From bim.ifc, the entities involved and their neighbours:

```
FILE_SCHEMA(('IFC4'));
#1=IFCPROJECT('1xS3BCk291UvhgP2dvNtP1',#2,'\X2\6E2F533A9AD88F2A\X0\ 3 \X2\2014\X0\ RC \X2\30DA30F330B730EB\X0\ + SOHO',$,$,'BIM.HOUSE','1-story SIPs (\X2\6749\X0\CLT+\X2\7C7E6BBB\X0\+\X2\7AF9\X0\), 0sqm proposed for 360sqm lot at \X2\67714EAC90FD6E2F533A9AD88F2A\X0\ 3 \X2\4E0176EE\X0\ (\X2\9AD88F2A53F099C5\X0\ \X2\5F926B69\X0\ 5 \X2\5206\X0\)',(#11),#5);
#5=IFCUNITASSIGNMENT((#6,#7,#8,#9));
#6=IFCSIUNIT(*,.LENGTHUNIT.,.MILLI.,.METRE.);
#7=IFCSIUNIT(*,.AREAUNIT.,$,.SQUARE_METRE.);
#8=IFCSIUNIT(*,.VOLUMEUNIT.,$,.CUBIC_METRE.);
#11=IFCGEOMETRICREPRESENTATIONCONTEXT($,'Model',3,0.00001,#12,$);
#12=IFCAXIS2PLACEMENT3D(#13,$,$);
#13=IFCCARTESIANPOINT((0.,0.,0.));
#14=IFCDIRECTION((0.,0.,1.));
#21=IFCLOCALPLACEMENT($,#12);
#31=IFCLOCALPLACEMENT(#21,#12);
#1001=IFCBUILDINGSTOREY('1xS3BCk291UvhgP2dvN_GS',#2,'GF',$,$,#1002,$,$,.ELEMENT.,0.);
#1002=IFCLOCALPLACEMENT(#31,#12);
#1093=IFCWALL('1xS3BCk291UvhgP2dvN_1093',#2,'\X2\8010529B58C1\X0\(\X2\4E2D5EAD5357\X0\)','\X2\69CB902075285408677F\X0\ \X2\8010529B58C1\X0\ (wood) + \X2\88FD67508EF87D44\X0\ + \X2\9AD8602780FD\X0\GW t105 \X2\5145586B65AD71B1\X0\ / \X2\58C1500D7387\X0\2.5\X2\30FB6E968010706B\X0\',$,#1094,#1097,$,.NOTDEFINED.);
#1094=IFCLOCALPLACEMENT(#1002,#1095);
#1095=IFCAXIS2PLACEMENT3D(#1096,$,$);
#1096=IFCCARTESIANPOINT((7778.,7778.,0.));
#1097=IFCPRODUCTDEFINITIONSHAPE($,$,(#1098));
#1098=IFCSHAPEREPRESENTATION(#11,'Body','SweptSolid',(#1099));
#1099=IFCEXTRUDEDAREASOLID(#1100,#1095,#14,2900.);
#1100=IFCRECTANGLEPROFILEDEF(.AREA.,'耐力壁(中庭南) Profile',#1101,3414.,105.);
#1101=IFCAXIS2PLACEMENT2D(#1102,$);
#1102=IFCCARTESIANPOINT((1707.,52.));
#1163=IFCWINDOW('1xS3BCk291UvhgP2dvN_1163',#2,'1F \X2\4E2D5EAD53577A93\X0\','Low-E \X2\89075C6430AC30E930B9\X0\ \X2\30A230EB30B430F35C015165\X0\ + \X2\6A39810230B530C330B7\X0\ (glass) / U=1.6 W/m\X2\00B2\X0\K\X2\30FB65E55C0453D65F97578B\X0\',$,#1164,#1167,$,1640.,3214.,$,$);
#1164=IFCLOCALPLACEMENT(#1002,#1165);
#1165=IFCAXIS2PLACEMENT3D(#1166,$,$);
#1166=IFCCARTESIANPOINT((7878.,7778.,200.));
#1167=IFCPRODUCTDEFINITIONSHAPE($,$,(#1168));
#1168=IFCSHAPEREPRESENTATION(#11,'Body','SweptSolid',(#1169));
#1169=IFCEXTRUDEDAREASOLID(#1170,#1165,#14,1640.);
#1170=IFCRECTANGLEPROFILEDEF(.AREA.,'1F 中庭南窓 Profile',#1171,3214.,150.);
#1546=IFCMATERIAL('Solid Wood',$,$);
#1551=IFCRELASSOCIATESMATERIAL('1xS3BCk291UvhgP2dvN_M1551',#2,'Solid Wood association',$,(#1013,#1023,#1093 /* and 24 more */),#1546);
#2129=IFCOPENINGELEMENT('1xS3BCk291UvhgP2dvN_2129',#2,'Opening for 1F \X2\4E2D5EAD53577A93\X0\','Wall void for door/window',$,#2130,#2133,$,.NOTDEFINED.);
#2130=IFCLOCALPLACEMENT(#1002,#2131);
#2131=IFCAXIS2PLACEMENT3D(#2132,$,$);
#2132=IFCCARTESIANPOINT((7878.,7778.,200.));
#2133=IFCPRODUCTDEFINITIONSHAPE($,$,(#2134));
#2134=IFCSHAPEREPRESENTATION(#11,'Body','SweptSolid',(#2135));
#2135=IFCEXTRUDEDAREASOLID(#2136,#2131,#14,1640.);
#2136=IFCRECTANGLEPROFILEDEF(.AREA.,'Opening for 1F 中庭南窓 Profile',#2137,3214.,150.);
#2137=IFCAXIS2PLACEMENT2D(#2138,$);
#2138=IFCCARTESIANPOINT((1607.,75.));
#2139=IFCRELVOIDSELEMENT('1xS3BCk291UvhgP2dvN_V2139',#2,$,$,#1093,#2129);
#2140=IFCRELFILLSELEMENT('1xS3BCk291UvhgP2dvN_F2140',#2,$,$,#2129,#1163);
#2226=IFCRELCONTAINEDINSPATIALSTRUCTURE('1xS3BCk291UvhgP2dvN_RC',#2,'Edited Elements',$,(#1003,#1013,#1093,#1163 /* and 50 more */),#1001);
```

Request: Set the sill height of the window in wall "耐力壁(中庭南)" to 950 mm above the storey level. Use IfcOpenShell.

```python
import numpy as np
import ifcopenshell
import ifcopenshell.api.geometry
import ifcopenshell.geom
import ifcopenshell.util.element
import ifcopenshell.util.placement
import ifcopenshell.util.shape
import ifcopenshell.util.unit

model = ifcopenshell.open("bim.ifc")
unit_scale = ifcopenshell.util.unit.calculate_unit_scale(model)

window = model.by_guid("1xS3BCk291UvhgP2dvN_1163")
opening = window.FillsVoids[0].RelatingOpeningElement
storey = ifcopenshell.util.element.get_container(window, ifc_class="IfcBuildingStorey")
level = ifcopenshell.util.placement.get_local_placement(storey.ObjectPlacement)[2, 3]

# The opening's origin need not be at the sill, so measure its lowest point.
shape = ifcopenshell.geom.create_shape(ifcopenshell.geom.settings(), opening)
bottom = ifcopenshell.util.shape.get_shape_bottom_elevation(shape, shape.geometry) / unit_scale
dz = level + 950.0 - bottom

shift = np.array([0.0, 0.0, dz])
# The window is not placed relative to its opening, so move both.
for product in (opening, window):
    matrix = ifcopenshell.util.placement.get_local_placement(product.ObjectPlacement)
    matrix[:3, 3] += shift
    ifcopenshell.api.geometry.edit_object_placement(model, product=product, matrix=matrix, is_si=False)

print(f"moved by {dz * unit_scale:+.3f} m")

model.write("bim_rev.ifc")
```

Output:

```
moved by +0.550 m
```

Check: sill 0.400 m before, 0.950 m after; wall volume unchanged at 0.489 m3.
